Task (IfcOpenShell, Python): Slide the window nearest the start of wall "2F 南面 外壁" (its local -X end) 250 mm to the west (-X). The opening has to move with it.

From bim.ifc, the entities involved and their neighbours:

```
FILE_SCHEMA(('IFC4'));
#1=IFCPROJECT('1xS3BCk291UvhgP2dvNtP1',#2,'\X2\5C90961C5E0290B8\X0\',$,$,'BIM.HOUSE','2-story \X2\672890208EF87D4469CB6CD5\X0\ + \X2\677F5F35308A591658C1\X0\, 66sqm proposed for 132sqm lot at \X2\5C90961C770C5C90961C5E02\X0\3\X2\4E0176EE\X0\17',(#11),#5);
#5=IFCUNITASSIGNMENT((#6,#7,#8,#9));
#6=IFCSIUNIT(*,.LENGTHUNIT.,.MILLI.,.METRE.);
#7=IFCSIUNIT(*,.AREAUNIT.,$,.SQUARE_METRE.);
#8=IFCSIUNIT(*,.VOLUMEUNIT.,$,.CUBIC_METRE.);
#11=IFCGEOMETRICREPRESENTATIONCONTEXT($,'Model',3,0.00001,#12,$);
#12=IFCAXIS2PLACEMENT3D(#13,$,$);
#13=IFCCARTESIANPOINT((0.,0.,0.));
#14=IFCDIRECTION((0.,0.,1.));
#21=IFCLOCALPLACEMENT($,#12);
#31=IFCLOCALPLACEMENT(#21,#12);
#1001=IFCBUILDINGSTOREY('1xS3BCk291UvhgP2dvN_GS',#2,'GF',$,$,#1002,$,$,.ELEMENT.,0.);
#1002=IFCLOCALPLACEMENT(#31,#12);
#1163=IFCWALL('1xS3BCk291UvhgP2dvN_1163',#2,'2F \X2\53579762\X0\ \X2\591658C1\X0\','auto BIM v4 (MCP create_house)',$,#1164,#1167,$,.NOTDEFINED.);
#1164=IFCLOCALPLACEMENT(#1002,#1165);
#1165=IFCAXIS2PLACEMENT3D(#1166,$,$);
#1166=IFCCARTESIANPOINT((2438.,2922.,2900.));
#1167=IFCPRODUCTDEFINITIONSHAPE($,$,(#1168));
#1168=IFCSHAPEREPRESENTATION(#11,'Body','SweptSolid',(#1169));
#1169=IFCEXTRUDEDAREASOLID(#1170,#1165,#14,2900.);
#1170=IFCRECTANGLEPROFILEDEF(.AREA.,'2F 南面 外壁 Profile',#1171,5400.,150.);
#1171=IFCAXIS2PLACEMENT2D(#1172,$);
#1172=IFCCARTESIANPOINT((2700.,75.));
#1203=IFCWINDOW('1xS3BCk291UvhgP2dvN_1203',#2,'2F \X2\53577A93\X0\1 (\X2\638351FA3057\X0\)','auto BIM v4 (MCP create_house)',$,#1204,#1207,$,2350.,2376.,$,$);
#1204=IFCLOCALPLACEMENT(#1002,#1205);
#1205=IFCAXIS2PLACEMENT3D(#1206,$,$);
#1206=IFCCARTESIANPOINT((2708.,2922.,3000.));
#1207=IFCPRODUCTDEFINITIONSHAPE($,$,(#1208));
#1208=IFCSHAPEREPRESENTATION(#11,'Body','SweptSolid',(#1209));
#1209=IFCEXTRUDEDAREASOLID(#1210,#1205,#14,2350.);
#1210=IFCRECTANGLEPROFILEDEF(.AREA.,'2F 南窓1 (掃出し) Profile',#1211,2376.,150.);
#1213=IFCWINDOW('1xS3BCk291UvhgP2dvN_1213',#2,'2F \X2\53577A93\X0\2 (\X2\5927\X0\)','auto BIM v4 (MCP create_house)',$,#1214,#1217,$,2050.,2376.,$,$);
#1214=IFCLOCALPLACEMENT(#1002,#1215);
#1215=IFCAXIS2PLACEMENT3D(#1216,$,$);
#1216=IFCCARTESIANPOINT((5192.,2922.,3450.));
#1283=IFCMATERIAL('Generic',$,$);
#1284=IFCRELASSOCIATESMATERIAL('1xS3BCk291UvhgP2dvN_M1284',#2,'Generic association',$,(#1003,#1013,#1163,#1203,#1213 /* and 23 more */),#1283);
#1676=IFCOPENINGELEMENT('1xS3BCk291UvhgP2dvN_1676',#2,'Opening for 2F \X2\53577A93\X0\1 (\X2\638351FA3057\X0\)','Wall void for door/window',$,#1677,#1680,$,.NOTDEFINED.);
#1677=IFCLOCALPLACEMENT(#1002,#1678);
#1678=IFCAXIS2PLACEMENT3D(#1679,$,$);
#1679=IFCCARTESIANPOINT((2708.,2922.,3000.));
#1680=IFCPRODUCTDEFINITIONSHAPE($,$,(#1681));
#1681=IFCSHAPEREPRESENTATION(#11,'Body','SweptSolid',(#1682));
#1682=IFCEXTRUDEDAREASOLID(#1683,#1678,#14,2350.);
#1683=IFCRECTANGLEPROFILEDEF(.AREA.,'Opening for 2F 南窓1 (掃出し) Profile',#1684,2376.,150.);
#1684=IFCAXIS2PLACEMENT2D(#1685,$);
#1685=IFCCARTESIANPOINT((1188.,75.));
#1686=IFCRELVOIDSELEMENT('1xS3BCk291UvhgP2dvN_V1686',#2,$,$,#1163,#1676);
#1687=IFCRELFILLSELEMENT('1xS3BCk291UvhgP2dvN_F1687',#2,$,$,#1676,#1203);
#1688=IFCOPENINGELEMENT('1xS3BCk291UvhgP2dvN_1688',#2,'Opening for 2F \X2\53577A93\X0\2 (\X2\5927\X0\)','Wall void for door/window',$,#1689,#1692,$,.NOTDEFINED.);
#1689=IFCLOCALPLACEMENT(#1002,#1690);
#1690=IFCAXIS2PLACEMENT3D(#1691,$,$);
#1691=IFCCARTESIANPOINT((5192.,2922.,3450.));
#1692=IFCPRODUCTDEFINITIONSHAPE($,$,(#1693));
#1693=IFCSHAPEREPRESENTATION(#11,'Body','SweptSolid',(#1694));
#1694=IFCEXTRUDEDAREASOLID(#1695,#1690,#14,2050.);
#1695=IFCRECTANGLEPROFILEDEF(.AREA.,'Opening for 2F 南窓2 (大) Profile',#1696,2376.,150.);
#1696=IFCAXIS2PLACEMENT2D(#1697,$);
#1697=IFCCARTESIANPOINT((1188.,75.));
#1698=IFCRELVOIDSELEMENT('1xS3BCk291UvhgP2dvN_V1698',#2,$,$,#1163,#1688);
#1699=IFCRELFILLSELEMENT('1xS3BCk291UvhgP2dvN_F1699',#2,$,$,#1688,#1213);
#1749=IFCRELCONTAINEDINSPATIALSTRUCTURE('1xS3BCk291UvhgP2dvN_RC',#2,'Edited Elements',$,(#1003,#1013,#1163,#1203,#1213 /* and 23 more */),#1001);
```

```python
import ifcopenshell
import ifcopenshell.api.geometry
import ifcopenshell.util.placement
import ifcopenshell.util.unit

model = ifcopenshell.open("bim.ifc")
unit_scale = ifcopenshell.util.unit.calculate_unit_scale(model)

window = model.by_guid("1xS3BCk291UvhgP2dvN_1203")
opening = window.FillsVoids[0].RelatingOpeningElement
wall = opening.VoidsElements[0].RelatingBuildingElement

wall_matrix = ifcopenshell.util.placement.get_local_placement(wall.ObjectPlacement)
shift = wall_matrix[:3, 0] * -0.25 / unit_scale
before = ifcopenshell.util.placement.get_local_placement(window.ObjectPlacement)[:3, 3].copy()

# The window is not placed relative to its opening, so move both.
for product in (opening, window):
    matrix = ifcopenshell.util.placement.get_local_placement(product.ObjectPlacement)
    matrix[:3, 3] += shift
    ifcopenshell.api.geometry.edit_object_placement(model, product=product, matrix=matrix, is_si=False)

after = ifcopenshell.util.placement.get_local_placement(window.ObjectPlacement)[:3, 3]
print("window moved by", (after - before).round(3) + 0.0)

model.write("bim_v2.ifc")
```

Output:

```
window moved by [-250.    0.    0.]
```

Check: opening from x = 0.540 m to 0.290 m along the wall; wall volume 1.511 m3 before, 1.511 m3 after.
